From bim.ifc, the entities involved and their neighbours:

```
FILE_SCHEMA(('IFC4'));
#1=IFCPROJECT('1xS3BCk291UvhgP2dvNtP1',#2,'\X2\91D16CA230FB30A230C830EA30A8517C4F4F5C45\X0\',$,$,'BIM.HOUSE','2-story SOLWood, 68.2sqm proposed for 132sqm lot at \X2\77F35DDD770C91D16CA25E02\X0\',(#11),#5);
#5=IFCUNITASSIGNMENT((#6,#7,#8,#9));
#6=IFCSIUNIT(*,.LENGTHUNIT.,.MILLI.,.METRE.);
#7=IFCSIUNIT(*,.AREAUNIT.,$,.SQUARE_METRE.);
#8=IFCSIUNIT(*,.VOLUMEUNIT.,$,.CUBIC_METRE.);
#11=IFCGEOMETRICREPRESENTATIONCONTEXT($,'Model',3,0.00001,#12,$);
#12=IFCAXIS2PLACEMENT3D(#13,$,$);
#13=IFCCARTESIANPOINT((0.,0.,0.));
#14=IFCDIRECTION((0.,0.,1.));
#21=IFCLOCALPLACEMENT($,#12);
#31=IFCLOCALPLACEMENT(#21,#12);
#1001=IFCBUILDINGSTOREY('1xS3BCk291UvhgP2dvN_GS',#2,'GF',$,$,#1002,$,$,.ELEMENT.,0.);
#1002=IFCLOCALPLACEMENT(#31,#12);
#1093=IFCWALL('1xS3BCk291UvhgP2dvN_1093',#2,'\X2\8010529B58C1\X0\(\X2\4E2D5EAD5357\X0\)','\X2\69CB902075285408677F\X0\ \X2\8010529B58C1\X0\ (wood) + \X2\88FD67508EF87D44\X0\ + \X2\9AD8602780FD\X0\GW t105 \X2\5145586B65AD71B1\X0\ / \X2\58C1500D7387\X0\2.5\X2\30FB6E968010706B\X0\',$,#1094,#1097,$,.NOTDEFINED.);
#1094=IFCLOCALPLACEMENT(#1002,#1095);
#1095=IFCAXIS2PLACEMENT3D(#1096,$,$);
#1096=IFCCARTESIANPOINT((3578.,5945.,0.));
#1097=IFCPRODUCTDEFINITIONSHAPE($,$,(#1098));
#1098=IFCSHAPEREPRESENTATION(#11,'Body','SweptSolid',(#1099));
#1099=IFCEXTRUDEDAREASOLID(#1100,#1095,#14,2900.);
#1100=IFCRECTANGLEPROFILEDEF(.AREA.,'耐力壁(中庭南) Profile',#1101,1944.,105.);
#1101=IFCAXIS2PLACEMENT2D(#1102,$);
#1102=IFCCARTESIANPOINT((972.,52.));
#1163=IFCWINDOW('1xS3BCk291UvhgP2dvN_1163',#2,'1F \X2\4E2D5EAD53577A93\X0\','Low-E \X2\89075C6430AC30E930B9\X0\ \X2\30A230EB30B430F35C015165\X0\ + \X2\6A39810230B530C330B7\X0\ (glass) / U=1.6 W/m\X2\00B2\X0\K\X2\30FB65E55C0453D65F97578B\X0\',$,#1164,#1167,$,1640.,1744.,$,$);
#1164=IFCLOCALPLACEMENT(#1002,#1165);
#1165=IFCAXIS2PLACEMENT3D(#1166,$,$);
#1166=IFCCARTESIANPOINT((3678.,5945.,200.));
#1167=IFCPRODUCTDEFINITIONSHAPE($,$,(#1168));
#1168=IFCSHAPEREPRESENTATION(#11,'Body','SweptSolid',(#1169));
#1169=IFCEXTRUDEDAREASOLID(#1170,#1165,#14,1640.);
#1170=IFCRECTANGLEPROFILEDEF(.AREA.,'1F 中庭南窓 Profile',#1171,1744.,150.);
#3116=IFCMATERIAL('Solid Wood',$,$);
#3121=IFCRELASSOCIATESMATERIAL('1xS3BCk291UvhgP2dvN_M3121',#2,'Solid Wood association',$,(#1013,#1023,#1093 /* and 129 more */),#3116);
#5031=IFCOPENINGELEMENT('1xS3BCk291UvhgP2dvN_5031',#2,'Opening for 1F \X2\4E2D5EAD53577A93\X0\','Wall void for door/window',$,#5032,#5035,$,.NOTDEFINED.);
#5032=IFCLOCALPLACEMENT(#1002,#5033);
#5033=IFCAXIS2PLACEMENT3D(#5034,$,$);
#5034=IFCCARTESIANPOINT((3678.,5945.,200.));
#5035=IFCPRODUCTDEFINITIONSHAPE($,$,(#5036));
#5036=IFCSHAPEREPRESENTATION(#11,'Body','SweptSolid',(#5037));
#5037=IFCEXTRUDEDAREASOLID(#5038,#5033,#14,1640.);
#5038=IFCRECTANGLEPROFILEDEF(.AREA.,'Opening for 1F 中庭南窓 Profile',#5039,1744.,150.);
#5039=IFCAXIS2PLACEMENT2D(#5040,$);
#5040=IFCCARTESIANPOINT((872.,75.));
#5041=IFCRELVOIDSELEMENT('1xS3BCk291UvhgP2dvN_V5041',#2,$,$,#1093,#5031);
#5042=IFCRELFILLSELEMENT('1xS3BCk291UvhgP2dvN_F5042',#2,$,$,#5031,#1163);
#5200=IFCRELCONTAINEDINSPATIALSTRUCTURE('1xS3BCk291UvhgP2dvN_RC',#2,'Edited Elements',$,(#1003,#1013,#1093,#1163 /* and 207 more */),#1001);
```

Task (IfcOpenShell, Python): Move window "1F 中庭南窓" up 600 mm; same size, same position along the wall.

```python
import numpy as np
import ifcopenshell
import ifcopenshell.api.geometry
import ifcopenshell.util.placement
import ifcopenshell.util.unit

model = ifcopenshell.open("bim.ifc")
unit_scale = ifcopenshell.util.unit.calculate_unit_scale(model)

window = model.by_guid("1xS3BCk291UvhgP2dvN_1163")
opening = window.FillsVoids[0].RelatingOpeningElement
dz = 0.6 / unit_scale

shift = np.array([0.0, 0.0, dz])
# The window is not placed relative to its opening, so move both.
for product in (opening, window):
    matrix = ifcopenshell.util.placement.get_local_placement(product.ObjectPlacement)
    matrix[:3, 3] += shift
    ifcopenshell.api.geometry.edit_object_placement(model, product=product, matrix=matrix, is_si=False)

print(f"moved by {dz * unit_scale:+.3f} m")

model.write("bim_edited.ifc")
```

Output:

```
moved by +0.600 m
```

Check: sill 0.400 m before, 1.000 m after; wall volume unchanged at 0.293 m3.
